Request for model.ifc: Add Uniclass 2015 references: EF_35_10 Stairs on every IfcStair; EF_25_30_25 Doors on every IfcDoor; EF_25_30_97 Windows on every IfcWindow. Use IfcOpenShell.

First a look at what the model holds.

```python
import ifcopenshell

model = ifcopenshell.open("model.ifc")
print(model.schema)
print("classifications:", [c.Name for c in model.by_type("IfcClassification")])
for ifc_class in ("IfcDoor", "IfcRoof", "IfcStair", "IfcWall", "IfcWindow"):
    print(ifc_class, len(model.by_type(ifc_class)))
```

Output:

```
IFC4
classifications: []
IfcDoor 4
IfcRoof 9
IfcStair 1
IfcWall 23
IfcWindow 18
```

```python
import ifcopenshell
import ifcopenshell.api.classification

model = ifcopenshell.open("model.ifc")

system = ifcopenshell.api.classification.add_classification(model, classification="Uniclass 2015")

codes = {
    "IfcStair": ("EF_35_10", "Stairs"),
    "IfcDoor": ("EF_25_30_25", "Doors"),
    "IfcWindow": ("EF_25_30_97", "Windows"),
}
for ifc_class, (code, name) in codes.items():
    products = model.by_type(ifc_class)
    ifcopenshell.api.classification.add_reference(
        model, products=products, classification=system, identification=code, name=name
    )
    print(code, len(products))

model.write("model-out.ifc")
```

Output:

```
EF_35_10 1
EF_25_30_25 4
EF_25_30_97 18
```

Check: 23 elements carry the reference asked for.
